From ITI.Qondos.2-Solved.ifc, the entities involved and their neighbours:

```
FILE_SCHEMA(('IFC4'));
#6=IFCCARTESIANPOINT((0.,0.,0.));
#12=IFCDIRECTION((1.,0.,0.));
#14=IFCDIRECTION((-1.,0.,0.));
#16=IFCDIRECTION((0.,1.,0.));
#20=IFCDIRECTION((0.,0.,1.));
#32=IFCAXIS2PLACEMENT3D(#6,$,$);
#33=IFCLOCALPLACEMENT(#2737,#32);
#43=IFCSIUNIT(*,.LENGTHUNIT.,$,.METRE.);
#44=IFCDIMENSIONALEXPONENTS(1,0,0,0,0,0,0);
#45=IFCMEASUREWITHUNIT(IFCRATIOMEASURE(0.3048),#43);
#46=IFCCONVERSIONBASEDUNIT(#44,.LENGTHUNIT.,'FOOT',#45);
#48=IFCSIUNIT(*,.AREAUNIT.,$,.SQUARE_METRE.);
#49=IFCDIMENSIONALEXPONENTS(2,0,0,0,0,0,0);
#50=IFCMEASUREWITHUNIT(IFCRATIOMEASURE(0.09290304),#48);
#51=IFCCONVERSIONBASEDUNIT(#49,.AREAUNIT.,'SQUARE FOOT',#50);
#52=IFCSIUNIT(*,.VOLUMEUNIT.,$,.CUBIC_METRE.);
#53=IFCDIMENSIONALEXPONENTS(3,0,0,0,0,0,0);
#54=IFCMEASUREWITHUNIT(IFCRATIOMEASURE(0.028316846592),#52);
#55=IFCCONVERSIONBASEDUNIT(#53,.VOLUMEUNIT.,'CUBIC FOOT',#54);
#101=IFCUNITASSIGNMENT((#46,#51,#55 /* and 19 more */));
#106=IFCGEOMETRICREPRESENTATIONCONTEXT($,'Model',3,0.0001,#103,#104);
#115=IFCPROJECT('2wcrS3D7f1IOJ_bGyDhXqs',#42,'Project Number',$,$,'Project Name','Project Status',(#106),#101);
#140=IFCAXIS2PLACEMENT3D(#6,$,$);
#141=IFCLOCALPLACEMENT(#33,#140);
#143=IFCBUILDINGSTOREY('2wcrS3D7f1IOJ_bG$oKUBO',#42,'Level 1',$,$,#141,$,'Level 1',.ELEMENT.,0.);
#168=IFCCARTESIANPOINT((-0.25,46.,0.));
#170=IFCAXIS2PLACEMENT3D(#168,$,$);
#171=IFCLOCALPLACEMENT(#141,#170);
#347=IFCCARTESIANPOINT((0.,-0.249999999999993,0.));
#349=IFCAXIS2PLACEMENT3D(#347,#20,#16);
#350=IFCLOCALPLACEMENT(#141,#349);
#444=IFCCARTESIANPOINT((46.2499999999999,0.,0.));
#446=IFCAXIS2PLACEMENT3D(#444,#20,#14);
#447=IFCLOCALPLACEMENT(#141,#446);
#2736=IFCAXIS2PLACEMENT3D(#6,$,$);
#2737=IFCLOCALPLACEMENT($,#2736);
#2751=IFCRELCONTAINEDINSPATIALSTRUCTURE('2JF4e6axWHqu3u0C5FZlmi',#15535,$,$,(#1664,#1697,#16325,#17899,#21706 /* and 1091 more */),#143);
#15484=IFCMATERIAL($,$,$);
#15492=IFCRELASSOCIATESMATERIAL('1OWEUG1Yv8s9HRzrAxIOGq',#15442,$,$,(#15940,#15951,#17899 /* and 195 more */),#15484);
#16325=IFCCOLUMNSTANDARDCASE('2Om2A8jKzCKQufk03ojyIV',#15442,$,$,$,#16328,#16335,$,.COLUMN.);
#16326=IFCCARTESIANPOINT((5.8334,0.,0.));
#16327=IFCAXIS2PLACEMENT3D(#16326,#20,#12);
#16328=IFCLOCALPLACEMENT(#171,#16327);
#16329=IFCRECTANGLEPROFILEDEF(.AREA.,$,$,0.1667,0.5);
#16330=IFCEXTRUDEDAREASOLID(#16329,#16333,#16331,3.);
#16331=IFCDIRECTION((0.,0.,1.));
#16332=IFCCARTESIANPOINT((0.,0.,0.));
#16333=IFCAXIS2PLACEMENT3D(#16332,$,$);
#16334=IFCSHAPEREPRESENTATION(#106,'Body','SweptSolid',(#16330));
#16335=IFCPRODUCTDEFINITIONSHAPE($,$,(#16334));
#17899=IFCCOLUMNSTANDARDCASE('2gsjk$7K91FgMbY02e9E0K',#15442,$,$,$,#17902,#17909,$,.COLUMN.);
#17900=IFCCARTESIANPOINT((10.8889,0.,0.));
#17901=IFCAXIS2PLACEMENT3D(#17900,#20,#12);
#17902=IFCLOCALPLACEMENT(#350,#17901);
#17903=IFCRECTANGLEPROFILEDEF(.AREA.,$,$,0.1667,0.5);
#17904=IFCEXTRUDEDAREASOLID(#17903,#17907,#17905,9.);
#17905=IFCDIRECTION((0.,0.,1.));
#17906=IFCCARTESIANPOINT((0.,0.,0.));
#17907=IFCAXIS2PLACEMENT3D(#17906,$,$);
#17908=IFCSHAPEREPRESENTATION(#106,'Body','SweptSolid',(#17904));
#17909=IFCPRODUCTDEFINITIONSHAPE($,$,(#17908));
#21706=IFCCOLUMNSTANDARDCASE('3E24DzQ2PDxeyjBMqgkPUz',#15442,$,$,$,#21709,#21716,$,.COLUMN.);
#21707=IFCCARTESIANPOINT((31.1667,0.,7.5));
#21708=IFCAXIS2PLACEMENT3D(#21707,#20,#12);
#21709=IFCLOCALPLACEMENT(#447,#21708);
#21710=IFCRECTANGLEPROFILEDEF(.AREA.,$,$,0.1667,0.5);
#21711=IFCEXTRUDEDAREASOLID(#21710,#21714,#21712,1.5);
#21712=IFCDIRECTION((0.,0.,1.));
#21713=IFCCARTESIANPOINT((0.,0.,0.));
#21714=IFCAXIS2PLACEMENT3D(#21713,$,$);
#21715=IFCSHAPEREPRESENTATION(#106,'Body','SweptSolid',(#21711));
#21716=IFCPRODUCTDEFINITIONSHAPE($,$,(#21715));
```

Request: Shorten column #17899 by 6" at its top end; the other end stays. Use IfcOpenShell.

```python
import ifcopenshell
import ifcopenshell.util.unit

model = ifcopenshell.open("ITI.Qondos.2-Solved.ifc")
unit_scale = ifcopenshell.util.unit.calculate_unit_scale(model)

member = model.by_guid("2gsjk$7K91FgMbY02e9E0K")
change = -6 * 0.0254 / unit_scale

# The extrusion runs towards the end named, so only its depth changes.
body = next(r for r in member.Representation.Representations if r.RepresentationIdentifier == "Body")
solid = body.Items[0]
old_length = solid.Depth
solid.Depth += change

print(f"length {old_length:g} -> {solid.Depth:g}")

model.write("ITI.Qondos.2-Solved_v2.ifc")
```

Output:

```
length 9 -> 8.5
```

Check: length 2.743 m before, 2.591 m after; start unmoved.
